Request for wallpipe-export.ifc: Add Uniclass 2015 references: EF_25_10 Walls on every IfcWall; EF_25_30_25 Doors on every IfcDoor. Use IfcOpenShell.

First a look at what the model holds.

```python
import ifcopenshell

model = ifcopenshell.open("wallpipe-export.ifc")
print(model.schema)
print("classifications:", [c.Name for c in model.by_type("IfcClassification")])
for ifc_class in ("IfcDoor", "IfcRoof", "IfcStair", "IfcWall", "IfcWindow"):
    print(ifc_class, len(model.by_type(ifc_class)))
```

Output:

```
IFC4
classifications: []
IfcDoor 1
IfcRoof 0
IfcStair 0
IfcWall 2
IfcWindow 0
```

```python
import ifcopenshell
import ifcopenshell.api.classification

model = ifcopenshell.open("wallpipe-export.ifc")

system = ifcopenshell.api.classification.add_classification(model, classification="Uniclass 2015")

codes = {
    "IfcWall": ("EF_25_10", "Walls"),
    "IfcDoor": ("EF_25_30_25", "Doors"),
}
for ifc_class, (code, name) in codes.items():
    products = model.by_type(ifc_class)
    ifcopenshell.api.classification.add_reference(
        model, products=products, classification=system, identification=code, name=name
    )
    print(code, len(products))

model.write("wallpipe-export_updated.ifc")
```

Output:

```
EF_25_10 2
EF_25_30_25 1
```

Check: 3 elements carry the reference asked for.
